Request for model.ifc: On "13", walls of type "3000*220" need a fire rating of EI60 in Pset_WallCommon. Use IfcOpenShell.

First a look at what the model holds.

```python
import ifcopenshell
import ifcopenshell.util.element

model = ifcopenshell.open("model.ifc")
print(model.schema)
storey = next(s for s in model.by_type("IfcBuildingStorey") if s.Name == "13")
walls = [e for e in ifcopenshell.util.element.get_decomposition(storey) if e.is_a("IfcWall")]
seen = {}
for e in walls:
    element_type = ifcopenshell.util.element.get_type(e)
    key = (element_type.Name if element_type != e and element_type else None, ifcopenshell.util.element.get_pset(e, "Pset_WallCommon", "FireRating"))
    seen[key] = seen.get(key, 0) + 1
for (name, value), count in sorted(seen.items(), key=str):
    print(count, "x", name, "|", value)
```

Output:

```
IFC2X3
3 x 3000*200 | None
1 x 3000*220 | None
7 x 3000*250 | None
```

```python
import ifcopenshell
import ifcopenshell.api.pset
import ifcopenshell.util.element

model = ifcopenshell.open("model.ifc")

storey = next(s for s in model.by_type("IfcBuildingStorey") if s.Name == "13")
walls = [e for e in ifcopenshell.util.element.get_decomposition(storey) if e.is_a("IfcWall")]

count = 0
for e in walls:
    element_type = ifcopenshell.util.element.get_type(e)
    if element_type in (None, e) or element_type.Name != "3000*220":
        continue
    found = ifcopenshell.util.element.get_pset(e, "Pset_WallCommon", should_inherit=False)
    if found:
        pset = model.by_id(found["id"])
        if len(ifcopenshell.util.element.get_elements_by_pset(pset)) > 1:
            pset = ifcopenshell.api.pset.unshare_pset(model, products=[e], pset=pset)[0]
    else:
        pset = ifcopenshell.api.pset.add_pset(model, product=e, name="Pset_WallCommon")
    ifcopenshell.api.pset.edit_pset(model, pset=pset, properties={"FireRating": "EI60"})
    count += 1

print(count, "walls updated")

model.write("model_edited.ifc")
```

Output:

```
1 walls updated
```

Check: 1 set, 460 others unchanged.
